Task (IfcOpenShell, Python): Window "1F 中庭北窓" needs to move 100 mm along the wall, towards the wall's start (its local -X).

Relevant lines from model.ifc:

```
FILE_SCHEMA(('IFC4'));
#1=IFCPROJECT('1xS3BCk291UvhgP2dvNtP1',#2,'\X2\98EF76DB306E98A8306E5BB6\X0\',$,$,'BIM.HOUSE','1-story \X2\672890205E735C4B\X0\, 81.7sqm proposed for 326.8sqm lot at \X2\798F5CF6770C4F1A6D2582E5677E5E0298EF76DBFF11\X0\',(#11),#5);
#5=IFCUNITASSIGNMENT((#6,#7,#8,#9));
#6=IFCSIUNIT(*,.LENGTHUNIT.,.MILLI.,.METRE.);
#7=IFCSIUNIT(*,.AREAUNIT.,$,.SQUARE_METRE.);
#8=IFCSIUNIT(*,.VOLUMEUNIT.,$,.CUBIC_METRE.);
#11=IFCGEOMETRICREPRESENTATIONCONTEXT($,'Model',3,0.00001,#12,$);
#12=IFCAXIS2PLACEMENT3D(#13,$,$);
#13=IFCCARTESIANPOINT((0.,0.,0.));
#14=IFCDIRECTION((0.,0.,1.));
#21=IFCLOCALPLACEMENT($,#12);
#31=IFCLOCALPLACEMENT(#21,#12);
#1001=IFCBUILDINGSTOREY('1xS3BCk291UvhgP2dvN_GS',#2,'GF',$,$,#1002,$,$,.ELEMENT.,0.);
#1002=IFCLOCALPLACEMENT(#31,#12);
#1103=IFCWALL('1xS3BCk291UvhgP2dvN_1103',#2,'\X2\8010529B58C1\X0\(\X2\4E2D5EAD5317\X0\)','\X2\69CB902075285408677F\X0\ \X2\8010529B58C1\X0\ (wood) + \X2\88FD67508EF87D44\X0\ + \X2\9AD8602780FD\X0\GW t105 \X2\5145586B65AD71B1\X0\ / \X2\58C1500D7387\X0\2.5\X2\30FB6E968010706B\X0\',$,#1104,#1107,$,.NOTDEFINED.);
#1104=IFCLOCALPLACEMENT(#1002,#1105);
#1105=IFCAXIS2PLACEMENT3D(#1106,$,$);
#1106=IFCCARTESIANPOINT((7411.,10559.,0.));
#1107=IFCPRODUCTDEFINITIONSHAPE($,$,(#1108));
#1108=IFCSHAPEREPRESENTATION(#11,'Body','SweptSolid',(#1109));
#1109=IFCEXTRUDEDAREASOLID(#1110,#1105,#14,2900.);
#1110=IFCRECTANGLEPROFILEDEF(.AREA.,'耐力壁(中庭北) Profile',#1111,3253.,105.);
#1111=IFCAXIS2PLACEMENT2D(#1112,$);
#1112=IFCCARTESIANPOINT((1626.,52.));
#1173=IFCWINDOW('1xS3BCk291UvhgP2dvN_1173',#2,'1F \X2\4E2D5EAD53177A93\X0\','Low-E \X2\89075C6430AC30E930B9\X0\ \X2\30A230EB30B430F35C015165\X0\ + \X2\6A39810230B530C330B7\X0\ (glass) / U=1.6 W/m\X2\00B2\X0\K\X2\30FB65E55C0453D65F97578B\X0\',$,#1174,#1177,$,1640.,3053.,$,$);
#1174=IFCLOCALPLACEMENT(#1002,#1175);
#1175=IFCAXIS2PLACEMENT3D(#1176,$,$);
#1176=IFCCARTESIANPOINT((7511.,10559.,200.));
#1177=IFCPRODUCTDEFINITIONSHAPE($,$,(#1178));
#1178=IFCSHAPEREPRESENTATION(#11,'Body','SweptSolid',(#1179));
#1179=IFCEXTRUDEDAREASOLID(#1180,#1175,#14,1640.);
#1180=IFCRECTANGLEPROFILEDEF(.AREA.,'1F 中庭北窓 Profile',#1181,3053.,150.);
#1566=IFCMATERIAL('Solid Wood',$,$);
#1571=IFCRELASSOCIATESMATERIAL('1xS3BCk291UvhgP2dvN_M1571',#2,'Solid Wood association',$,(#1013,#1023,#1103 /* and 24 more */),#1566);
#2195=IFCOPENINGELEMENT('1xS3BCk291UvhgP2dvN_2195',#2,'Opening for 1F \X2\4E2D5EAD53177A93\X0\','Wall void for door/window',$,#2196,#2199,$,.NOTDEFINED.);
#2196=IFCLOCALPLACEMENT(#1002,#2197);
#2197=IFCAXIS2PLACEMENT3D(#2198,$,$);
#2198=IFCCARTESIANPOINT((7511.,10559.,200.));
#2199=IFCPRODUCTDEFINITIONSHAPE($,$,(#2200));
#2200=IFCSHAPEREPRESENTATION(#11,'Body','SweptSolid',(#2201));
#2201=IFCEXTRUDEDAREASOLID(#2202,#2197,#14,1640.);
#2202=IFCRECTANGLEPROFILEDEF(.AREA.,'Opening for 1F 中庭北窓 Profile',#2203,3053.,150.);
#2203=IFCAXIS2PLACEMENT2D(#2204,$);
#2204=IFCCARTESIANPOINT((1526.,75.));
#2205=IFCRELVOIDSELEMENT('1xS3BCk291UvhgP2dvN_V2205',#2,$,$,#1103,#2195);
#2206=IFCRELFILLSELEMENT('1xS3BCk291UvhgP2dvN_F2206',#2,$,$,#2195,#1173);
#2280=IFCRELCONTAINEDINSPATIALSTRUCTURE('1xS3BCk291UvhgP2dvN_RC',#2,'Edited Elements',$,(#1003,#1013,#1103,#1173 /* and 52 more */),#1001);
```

```python
import ifcopenshell
import ifcopenshell.api.geometry
import ifcopenshell.util.placement

model = ifcopenshell.open("model.ifc")

window = model.by_id(1173)
opening = window.FillsVoids[0].RelatingOpeningElement
wall = opening.VoidsElements[0].RelatingBuildingElement

wall_matrix = ifcopenshell.util.placement.get_local_placement(wall.ObjectPlacement)
shift = wall_matrix[:3, 0] * -100.0
before = ifcopenshell.util.placement.get_local_placement(window.ObjectPlacement)[:3, 3].copy()

# The window is not placed relative to its opening, so move both.
for product in (opening, window):
    matrix = ifcopenshell.util.placement.get_local_placement(product.ObjectPlacement)
    matrix[:3, 3] += shift
    ifcopenshell.api.geometry.edit_object_placement(model, product=product, matrix=matrix, is_si=False)

after = ifcopenshell.util.placement.get_local_placement(window.ObjectPlacement)[:3, 3]
print("window moved by", (after - before).round(3) + 0.0)

model.write("model_v2.ifc")
```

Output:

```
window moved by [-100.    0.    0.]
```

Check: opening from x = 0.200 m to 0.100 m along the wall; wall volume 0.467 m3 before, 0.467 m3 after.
